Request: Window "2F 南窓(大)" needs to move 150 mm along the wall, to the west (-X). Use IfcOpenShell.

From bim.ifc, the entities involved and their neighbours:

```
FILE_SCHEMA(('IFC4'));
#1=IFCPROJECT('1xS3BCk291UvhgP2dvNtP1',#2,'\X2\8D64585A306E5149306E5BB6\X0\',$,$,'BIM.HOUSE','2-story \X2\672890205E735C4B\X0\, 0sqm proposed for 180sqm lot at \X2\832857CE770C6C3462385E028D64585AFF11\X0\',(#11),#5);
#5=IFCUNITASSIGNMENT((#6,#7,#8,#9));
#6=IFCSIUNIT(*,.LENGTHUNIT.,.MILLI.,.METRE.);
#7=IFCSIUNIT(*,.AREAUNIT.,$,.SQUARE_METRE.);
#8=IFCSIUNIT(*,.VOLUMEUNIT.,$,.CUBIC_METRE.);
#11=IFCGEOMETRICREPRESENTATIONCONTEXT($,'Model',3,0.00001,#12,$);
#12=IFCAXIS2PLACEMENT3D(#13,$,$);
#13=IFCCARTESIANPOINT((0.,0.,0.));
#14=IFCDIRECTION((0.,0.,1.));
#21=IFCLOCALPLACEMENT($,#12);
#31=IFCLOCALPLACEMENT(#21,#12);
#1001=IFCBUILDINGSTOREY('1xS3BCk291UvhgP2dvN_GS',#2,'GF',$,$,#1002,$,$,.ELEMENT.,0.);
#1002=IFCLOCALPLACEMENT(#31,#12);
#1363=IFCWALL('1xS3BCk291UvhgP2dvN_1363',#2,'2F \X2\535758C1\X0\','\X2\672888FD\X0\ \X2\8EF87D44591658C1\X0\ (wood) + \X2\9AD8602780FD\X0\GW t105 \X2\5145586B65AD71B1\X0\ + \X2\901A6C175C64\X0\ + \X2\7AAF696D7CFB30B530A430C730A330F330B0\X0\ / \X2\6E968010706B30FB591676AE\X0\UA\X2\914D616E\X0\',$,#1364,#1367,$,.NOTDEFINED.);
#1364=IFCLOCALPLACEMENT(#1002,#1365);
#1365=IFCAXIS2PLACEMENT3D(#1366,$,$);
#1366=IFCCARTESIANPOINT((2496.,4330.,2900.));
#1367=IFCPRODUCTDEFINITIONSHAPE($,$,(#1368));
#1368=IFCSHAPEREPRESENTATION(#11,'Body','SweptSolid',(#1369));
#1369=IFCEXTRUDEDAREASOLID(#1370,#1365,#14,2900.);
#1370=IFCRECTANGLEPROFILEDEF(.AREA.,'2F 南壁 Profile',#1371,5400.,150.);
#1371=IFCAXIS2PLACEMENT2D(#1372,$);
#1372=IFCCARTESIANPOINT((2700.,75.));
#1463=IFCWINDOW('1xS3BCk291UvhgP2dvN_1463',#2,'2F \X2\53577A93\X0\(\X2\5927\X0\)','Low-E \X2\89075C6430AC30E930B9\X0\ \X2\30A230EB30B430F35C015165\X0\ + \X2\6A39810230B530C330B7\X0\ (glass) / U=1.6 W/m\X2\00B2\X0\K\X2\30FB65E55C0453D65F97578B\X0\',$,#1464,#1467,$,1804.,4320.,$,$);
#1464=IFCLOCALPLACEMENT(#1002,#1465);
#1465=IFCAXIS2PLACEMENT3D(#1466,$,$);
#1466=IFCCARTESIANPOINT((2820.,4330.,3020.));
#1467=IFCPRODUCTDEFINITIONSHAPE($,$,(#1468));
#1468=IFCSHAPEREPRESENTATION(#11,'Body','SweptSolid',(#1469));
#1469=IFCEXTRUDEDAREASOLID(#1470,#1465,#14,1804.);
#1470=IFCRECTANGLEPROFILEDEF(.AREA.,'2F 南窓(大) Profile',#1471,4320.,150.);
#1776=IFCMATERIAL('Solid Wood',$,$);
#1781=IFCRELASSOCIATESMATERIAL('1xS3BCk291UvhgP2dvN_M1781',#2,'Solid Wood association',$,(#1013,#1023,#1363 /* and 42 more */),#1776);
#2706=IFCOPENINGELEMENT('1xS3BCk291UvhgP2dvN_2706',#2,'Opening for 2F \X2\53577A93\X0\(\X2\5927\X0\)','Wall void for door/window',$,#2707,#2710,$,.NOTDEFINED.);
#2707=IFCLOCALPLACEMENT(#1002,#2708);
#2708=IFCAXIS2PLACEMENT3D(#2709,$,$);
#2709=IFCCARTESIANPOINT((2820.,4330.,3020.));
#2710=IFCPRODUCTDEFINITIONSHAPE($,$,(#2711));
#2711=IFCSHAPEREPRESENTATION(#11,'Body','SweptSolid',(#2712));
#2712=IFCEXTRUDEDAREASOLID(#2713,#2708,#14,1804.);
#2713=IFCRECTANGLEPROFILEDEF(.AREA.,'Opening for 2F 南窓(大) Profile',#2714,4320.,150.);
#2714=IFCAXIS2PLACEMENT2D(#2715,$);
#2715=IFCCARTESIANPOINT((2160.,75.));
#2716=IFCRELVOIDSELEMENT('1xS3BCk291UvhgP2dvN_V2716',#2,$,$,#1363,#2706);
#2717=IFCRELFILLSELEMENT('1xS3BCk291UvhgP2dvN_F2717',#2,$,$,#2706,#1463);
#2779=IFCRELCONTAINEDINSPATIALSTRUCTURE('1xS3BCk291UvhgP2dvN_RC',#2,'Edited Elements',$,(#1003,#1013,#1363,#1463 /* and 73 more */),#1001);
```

```python
import ifcopenshell
import ifcopenshell.api.geometry
import ifcopenshell.util.placement
import ifcopenshell.util.unit

model = ifcopenshell.open("bim.ifc")
unit_scale = ifcopenshell.util.unit.calculate_unit_scale(model)

window = model.by_id(1463)
opening = window.FillsVoids[0].RelatingOpeningElement
wall = opening.VoidsElements[0].RelatingBuildingElement

wall_matrix = ifcopenshell.util.placement.get_local_placement(wall.ObjectPlacement)
shift = wall_matrix[:3, 0] * -0.15 / unit_scale
before = ifcopenshell.util.placement.get_local_placement(window.ObjectPlacement)[:3, 3].copy()

# The window is not placed relative to its opening, so move both.
for product in (opening, window):
    matrix = ifcopenshell.util.placement.get_local_placement(product.ObjectPlacement)
    matrix[:3, 3] += shift
    ifcopenshell.api.geometry.edit_object_placement(model, product=product, matrix=matrix, is_si=False)

after = ifcopenshell.util.placement.get_local_placement(window.ObjectPlacement)[:3, 3]
print("window moved by", (after - before).round(3) + 0.0)

model.write("bim_v2.ifc")
```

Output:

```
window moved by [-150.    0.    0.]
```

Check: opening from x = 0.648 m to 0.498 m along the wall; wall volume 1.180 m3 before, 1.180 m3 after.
